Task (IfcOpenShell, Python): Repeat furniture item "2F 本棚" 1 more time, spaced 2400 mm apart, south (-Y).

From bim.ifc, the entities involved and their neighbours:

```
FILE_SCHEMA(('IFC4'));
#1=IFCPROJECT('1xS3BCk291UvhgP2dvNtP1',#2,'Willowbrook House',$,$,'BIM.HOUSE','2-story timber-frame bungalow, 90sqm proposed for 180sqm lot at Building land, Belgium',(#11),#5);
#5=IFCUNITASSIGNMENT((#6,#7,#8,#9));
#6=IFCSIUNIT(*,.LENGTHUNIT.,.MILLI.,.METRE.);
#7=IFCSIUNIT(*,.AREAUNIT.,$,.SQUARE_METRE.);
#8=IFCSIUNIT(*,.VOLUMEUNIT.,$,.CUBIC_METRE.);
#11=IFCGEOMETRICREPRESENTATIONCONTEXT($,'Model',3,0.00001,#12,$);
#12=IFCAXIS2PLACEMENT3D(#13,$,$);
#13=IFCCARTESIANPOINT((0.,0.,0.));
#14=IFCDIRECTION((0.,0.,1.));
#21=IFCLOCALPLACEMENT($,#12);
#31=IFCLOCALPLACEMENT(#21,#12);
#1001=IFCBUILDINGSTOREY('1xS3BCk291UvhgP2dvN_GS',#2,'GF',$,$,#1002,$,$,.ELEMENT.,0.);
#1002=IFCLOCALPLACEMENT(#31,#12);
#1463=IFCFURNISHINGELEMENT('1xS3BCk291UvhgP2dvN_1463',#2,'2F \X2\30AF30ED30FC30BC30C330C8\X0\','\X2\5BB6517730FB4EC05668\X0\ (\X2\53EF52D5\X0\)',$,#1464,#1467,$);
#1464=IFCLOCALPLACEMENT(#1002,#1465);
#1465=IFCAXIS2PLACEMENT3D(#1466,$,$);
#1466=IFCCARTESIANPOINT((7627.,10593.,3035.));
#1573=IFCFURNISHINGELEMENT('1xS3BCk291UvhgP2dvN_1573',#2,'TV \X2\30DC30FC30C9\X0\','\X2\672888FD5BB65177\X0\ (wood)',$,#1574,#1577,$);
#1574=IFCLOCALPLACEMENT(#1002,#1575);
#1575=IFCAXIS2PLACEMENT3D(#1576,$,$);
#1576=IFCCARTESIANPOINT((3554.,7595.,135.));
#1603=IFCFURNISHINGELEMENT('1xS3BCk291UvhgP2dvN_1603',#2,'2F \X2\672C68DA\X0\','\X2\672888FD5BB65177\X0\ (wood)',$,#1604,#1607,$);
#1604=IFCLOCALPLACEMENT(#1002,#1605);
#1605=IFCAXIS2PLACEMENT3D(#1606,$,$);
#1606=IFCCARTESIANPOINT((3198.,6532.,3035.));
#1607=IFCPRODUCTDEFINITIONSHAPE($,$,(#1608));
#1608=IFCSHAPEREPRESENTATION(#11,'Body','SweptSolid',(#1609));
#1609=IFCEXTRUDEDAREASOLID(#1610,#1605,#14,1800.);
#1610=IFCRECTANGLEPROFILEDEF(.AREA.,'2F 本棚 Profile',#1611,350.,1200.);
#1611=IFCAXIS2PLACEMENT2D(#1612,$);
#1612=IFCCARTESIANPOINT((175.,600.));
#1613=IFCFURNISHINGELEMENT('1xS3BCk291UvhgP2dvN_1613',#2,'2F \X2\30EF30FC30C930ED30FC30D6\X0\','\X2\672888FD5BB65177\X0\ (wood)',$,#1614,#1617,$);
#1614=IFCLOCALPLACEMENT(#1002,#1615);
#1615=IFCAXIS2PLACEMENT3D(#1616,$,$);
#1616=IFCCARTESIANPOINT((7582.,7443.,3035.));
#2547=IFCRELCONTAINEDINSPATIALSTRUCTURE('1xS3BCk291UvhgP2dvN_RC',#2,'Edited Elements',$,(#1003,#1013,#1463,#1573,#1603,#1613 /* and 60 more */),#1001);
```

```python
import numpy as np
import ifcopenshell
import ifcopenshell.api.geometry
import ifcopenshell.api.root
import ifcopenshell.util.element
import ifcopenshell.util.placement
import ifcopenshell.util.unit

model = ifcopenshell.open("bim.ifc")
unit_scale = ifcopenshell.util.unit.calculate_unit_scale(model)


def reuse_history(source, copy):
    """copy_class also copies each property set's owner history, people and application; keep the originals."""
    for rel in copy.IsDefinedBy:
        if rel.is_a("IfcRelDefinesByProperties") and (history := rel.RelatingPropertyDefinition.OwnerHistory):
            rel.RelatingPropertyDefinition.OwnerHistory = source.OwnerHistory
            ifcopenshell.util.element.remove_deep2(model, history)


source = model.by_guid("1xS3BCk291UvhgP2dvN_1603")
base = ifcopenshell.util.placement.get_local_placement(source.ObjectPlacement)
step = np.array([0.0, -1.0, 0.0]) * 2.4 / unit_scale

for i in range(1, 2):
    copy = ifcopenshell.api.root.copy_class(model, product=source)
    copy.Representation = ifcopenshell.util.element.copy_deep(
        model, source.Representation, exclude=["IfcGeometricRepresentationContext", "IfcRepresentationMap"]
    )
    reuse_history(source, copy)
    matrix = base.copy()
    matrix[:3, 3] += i * step
    print("added at", matrix[:3, 3].round(3) + 0.0)
    ifcopenshell.api.geometry.edit_object_placement(model, product=copy, matrix=matrix, is_si=False)

model.write("bim_rev.ifc")
```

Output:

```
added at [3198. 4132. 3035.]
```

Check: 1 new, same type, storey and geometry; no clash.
